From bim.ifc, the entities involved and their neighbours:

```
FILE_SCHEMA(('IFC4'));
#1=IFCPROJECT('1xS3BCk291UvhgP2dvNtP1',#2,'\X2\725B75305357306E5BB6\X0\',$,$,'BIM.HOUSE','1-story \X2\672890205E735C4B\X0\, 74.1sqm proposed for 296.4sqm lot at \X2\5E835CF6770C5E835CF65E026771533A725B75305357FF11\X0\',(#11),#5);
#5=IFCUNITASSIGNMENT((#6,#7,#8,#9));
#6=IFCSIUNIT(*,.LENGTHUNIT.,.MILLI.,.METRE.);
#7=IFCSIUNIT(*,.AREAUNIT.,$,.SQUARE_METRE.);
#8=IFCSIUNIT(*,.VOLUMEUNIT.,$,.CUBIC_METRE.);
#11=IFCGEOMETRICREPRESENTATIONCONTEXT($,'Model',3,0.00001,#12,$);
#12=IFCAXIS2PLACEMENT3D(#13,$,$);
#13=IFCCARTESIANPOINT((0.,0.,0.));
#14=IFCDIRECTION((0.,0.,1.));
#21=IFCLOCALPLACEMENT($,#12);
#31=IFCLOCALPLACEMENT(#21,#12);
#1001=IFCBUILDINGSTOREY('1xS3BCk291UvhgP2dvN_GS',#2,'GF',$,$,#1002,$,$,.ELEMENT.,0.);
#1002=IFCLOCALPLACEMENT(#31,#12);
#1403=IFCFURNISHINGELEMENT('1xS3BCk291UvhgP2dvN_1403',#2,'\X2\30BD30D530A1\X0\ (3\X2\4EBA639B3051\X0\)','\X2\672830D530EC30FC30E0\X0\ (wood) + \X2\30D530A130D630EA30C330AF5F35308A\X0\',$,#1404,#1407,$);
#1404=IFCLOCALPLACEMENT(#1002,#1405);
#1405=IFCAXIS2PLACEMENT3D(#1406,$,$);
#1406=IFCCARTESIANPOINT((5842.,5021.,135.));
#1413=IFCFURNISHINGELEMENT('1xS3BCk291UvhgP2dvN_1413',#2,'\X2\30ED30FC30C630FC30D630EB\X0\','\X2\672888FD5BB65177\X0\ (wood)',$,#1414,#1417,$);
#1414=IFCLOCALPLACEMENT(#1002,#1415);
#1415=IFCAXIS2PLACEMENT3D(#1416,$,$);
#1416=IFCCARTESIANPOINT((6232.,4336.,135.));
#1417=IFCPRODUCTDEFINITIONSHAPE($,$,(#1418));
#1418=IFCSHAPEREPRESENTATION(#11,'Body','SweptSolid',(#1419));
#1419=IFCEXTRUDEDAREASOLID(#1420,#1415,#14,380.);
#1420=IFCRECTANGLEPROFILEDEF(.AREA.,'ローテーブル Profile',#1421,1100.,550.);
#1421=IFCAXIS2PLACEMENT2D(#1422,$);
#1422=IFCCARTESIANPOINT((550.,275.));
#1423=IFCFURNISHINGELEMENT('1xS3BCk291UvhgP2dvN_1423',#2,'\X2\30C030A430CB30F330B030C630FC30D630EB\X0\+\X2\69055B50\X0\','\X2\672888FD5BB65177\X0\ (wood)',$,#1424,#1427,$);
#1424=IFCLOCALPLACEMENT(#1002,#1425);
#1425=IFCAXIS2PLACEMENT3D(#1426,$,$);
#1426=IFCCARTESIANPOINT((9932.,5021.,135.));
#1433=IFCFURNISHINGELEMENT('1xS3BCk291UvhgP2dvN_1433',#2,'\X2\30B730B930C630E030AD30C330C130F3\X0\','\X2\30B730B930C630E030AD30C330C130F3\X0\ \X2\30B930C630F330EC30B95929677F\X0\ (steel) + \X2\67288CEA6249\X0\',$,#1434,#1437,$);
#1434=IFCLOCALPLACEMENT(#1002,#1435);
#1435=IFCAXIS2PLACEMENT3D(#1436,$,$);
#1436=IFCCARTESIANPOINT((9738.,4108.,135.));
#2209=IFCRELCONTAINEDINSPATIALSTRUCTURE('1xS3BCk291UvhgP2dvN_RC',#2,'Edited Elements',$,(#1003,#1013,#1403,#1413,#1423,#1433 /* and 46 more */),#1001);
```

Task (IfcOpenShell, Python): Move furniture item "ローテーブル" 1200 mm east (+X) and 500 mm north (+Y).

```python
import ifcopenshell
import ifcopenshell.api.geometry
import ifcopenshell.util.placement
import ifcopenshell.util.unit

model = ifcopenshell.open("bim.ifc")
unit_scale = ifcopenshell.util.unit.calculate_unit_scale(model)

item = model.by_id(1413)
matrix = ifcopenshell.util.placement.get_local_placement(item.ObjectPlacement)
matrix[0, 3] += 1.2 / unit_scale
matrix[1, 3] += 0.5 / unit_scale
ifcopenshell.api.geometry.edit_object_placement(model, product=item, matrix=matrix, is_si=False)

print(ifcopenshell.util.placement.get_local_placement(item.ObjectPlacement).round(3) + 0.0)

model.write("bim_updated.ifc")
```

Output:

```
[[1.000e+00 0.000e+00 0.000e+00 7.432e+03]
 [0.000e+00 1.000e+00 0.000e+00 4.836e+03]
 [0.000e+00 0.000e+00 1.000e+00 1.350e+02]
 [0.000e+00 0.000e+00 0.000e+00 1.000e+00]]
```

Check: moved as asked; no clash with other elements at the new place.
